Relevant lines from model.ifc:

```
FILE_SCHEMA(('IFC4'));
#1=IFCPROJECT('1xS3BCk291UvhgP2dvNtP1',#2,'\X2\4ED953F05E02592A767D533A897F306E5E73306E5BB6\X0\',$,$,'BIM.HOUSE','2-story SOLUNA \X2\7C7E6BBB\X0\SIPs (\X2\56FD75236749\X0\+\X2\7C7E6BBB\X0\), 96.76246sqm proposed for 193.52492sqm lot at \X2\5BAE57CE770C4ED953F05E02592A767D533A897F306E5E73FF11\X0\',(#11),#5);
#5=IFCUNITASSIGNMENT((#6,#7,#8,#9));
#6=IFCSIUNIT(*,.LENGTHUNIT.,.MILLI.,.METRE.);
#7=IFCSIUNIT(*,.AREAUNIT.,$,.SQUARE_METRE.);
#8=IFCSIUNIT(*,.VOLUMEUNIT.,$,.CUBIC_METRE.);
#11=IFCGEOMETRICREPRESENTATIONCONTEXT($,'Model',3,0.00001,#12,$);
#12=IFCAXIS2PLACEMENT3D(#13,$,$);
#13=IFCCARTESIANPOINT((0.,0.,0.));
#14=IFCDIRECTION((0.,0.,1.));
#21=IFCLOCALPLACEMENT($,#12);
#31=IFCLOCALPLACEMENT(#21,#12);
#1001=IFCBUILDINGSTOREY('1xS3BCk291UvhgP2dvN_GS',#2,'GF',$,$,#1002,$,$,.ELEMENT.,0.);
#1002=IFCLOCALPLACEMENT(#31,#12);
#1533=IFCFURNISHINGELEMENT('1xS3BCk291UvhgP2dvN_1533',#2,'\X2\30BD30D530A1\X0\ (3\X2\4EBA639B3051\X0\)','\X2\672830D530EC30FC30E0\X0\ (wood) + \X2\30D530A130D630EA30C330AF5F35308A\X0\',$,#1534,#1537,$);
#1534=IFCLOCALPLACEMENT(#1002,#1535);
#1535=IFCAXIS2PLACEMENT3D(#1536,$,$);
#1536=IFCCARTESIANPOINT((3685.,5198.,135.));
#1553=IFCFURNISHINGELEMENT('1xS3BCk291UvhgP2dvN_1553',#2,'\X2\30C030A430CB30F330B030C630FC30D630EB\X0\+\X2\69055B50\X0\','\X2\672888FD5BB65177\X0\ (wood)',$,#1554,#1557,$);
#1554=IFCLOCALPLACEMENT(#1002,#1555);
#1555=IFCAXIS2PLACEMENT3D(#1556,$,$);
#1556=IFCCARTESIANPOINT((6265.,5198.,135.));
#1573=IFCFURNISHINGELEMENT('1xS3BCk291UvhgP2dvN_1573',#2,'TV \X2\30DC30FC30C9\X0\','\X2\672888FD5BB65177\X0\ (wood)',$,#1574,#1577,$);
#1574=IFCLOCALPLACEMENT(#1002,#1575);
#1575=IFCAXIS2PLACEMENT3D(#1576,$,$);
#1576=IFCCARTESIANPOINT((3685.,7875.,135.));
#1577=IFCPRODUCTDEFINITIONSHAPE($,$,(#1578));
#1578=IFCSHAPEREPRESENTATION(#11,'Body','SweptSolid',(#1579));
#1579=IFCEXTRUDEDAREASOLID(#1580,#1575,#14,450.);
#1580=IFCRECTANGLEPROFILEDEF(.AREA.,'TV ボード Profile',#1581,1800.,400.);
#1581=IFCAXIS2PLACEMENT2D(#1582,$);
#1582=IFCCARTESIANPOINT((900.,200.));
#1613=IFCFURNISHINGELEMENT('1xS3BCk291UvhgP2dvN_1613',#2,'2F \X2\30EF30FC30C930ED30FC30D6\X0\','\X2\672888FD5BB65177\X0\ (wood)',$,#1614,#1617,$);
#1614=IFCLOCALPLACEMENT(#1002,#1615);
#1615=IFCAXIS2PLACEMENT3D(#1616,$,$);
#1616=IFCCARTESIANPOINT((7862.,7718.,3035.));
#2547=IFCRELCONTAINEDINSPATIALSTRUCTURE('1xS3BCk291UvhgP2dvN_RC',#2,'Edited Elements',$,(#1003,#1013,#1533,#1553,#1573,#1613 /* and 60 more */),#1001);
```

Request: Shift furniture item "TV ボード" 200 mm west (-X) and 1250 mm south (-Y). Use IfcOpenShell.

```python
import ifcopenshell
import ifcopenshell.api.geometry
import ifcopenshell.util.placement

model = ifcopenshell.open("model.ifc")

item = model.by_guid("1xS3BCk291UvhgP2dvN_1573")
matrix = ifcopenshell.util.placement.get_local_placement(item.ObjectPlacement)
matrix[0, 3] -= 200.0
matrix[1, 3] -= 1250.0
ifcopenshell.api.geometry.edit_object_placement(model, product=item, matrix=matrix, is_si=False)

print(ifcopenshell.util.placement.get_local_placement(item.ObjectPlacement).round(3) + 0.0)

model.write("model_rev.ifc")
```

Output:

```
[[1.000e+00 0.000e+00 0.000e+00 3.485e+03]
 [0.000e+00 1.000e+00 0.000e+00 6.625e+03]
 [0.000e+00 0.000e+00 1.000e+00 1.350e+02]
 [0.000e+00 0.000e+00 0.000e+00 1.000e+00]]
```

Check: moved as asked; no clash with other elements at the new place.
